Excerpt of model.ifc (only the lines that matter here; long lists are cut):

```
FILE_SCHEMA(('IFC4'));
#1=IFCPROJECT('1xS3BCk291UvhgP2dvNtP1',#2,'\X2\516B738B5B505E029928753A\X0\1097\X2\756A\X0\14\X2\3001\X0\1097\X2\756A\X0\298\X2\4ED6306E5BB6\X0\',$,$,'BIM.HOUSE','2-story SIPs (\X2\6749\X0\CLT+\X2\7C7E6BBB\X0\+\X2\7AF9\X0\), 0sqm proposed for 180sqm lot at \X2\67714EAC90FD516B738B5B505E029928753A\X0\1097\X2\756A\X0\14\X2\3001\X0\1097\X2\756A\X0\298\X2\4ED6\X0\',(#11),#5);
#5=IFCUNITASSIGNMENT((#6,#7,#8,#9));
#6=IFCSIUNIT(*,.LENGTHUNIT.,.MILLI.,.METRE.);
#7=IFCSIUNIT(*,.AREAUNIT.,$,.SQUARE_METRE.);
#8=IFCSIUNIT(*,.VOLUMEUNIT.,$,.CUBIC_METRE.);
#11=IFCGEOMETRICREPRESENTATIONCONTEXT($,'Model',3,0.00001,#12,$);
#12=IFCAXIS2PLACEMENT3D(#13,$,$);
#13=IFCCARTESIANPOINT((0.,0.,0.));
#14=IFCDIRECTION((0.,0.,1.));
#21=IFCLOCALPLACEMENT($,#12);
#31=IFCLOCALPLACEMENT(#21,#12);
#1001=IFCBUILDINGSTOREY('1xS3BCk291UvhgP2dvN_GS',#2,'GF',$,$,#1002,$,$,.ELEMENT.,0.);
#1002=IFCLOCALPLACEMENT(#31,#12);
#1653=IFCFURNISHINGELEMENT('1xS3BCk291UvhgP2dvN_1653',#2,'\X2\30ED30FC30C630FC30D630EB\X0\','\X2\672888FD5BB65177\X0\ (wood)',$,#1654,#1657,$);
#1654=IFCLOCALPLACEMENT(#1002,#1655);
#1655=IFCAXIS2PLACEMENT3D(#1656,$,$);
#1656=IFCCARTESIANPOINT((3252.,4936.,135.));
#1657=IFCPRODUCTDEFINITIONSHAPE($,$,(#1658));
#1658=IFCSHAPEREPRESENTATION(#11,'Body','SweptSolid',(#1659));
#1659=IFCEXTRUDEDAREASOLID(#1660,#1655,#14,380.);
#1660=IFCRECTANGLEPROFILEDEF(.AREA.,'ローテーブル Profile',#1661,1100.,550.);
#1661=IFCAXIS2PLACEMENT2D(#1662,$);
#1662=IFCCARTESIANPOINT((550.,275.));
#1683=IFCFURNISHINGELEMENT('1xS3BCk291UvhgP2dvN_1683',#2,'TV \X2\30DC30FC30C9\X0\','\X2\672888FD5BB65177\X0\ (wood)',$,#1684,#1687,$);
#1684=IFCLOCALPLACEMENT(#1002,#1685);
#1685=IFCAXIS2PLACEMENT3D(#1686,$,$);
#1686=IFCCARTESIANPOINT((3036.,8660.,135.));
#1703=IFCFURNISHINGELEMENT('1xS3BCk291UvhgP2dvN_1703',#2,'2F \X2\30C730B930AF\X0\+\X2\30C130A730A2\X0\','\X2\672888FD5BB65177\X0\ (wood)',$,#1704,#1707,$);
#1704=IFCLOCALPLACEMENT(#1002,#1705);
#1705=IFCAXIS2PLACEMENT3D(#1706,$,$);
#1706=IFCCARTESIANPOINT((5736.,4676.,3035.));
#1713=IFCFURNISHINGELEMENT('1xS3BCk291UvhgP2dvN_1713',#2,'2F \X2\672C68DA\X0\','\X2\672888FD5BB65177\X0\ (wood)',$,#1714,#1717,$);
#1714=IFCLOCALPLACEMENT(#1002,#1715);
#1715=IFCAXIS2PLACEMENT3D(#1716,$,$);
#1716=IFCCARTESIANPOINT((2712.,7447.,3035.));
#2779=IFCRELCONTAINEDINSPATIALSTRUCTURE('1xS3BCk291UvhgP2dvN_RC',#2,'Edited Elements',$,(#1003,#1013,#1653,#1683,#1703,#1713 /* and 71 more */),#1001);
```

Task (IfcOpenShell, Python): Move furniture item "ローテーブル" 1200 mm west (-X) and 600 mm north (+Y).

```python
import ifcopenshell
import ifcopenshell.api.geometry
import ifcopenshell.util.placement

model = ifcopenshell.open("model.ifc")

item = model.by_guid("1xS3BCk291UvhgP2dvN_1653")
matrix = ifcopenshell.util.placement.get_local_placement(item.ObjectPlacement)
matrix[0, 3] -= 1200.0
matrix[1, 3] += 600.0
ifcopenshell.api.geometry.edit_object_placement(model, product=item, matrix=matrix, is_si=False)

print(ifcopenshell.util.placement.get_local_placement(item.ObjectPlacement).round(3) + 0.0)

model.write("model-out.ifc")
```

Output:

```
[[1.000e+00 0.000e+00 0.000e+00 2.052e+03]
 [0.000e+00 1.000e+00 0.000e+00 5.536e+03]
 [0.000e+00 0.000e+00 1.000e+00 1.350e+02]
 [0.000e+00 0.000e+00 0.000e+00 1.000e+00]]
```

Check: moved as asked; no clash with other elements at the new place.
